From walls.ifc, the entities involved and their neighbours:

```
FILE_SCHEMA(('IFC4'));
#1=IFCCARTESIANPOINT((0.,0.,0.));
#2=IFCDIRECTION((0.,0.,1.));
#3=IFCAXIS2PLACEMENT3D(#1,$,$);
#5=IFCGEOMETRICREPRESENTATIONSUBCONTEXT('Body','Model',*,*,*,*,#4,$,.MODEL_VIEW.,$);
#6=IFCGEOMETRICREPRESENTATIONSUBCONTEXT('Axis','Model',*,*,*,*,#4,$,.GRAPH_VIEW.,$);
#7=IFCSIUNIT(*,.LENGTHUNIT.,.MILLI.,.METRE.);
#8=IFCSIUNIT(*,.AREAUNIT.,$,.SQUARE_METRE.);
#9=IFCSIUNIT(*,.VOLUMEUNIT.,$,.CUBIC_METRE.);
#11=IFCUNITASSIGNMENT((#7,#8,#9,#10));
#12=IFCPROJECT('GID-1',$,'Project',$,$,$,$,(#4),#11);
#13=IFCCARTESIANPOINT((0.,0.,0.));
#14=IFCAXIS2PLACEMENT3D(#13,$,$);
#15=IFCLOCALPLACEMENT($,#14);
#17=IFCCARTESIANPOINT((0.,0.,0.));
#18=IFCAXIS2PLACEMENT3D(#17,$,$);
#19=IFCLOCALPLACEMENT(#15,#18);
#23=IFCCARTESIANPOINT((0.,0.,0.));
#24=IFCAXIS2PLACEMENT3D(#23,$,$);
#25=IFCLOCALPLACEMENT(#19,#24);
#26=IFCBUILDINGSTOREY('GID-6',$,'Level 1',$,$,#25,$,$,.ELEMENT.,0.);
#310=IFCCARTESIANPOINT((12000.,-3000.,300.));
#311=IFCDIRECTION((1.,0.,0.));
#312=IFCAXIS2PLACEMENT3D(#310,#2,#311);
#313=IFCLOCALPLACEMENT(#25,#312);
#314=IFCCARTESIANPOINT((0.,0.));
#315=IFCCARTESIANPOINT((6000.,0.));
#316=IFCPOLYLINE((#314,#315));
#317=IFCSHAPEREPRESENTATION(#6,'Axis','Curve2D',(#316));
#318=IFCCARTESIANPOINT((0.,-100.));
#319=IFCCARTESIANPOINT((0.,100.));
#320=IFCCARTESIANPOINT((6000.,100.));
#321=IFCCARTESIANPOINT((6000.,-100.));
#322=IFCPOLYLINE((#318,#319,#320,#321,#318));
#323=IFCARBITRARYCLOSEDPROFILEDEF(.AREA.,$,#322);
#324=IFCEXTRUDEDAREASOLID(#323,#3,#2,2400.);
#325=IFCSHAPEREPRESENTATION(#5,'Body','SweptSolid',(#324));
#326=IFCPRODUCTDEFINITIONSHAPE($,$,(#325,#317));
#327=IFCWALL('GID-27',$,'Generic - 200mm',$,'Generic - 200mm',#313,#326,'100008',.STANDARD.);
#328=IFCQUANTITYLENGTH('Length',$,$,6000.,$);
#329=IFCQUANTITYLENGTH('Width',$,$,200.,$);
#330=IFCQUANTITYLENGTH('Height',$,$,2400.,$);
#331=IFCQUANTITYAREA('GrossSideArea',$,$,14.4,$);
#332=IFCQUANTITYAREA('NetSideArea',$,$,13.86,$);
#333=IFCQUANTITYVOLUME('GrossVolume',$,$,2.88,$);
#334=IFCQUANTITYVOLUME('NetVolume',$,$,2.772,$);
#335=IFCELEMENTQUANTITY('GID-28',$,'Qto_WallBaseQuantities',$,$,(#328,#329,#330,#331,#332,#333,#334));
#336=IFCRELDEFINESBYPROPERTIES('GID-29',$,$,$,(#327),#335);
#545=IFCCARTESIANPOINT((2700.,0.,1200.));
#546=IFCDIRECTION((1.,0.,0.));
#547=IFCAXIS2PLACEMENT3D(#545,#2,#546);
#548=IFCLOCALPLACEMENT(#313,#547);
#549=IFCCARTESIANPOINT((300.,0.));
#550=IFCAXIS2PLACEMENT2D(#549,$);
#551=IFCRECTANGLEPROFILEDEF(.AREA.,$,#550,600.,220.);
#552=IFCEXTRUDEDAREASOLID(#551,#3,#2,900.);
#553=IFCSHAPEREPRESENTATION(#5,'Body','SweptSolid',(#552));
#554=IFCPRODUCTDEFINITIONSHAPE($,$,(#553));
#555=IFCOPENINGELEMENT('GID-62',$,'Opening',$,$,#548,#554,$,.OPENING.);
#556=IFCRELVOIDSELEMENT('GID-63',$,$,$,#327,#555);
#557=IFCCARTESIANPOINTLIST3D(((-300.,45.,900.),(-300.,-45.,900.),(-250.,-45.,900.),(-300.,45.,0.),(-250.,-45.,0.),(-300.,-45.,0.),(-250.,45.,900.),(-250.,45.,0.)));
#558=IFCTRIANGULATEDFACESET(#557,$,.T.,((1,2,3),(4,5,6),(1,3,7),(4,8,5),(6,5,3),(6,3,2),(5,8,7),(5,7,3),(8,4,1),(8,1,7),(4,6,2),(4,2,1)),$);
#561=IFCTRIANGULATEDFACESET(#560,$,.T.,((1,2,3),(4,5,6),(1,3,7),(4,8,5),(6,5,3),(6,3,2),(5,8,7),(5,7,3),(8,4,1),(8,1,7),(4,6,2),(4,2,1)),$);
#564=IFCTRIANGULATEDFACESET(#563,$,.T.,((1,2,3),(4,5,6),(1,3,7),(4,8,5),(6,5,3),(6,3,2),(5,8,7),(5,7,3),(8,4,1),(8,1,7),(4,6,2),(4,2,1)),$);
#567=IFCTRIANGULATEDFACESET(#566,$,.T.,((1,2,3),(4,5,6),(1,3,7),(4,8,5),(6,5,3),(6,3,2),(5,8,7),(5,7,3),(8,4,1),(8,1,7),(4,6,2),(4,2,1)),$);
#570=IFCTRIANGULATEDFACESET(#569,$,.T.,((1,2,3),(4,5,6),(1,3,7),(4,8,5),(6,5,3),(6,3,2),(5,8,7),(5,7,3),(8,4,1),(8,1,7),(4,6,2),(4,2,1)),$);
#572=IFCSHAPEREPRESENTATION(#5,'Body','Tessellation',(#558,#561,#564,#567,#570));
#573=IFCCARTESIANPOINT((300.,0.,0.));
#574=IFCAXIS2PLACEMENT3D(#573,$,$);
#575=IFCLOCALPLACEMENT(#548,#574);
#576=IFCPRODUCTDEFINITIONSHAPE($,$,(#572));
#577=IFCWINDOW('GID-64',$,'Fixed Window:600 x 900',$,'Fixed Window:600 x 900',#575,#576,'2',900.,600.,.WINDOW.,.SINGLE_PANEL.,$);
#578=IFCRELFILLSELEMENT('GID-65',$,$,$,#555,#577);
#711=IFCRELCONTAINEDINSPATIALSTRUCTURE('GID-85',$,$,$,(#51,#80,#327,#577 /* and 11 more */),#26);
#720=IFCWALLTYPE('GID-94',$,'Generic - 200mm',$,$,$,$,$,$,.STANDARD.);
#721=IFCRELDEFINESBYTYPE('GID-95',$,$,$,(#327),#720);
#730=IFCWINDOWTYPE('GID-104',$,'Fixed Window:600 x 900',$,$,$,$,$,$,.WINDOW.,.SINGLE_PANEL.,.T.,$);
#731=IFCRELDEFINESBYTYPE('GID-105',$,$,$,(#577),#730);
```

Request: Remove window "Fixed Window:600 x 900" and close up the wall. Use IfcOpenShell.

```python
import ifcopenshell
import ifcopenshell.api.feature
import ifcopenshell.api.pset
import ifcopenshell.api.root
import ifcopenshell.geom
import ifcopenshell.util.element
import ifcopenshell.util.shape
import ifcopenshell.util.unit

model = ifcopenshell.open("walls.ifc")
area_scale = ifcopenshell.util.unit.calculate_unit_scale(model, "AREAUNIT")
volume_scale = ifcopenshell.util.unit.calculate_unit_scale(model, "VOLUMEUNIT")
settings = ifcopenshell.geom.settings()


def volume(element):
    """Net volume in cubic metres, openings subtracted."""
    shape = ifcopenshell.geom.create_shape(settings, element)
    return ifcopenshell.util.shape.get_volume(shape.geometry)


window = model.by_guid("GID-64")
opening = window.FillsVoids[0].RelatingOpeningElement
wall = opening.VoidsElements[0].RelatingBuildingElement
before = volume(wall)

ifcopenshell.api.root.remove_product(model, product=window)
ifcopenshell.api.feature.remove_feature(model, feature=opening)

after = volume(wall)
thickness = 0.2  # wall thickness in metres

# Update the wall's stored quantities.
qto = model.by_id(ifcopenshell.util.element.get_pset(wall, "Qto_WallBaseQuantities", should_inherit=False)["id"])
ifcopenshell.api.pset.edit_qto(model, qto=qto, properties={
    "NetSideArea": after / thickness / area_scale,
    "NetVolume": after / volume_scale,
})

print(f"wall volume {before:.3f} -> {after:.3f} m3")

model.write("walls-out.ifc")
```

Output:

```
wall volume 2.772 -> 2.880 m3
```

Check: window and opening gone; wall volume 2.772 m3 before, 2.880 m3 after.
